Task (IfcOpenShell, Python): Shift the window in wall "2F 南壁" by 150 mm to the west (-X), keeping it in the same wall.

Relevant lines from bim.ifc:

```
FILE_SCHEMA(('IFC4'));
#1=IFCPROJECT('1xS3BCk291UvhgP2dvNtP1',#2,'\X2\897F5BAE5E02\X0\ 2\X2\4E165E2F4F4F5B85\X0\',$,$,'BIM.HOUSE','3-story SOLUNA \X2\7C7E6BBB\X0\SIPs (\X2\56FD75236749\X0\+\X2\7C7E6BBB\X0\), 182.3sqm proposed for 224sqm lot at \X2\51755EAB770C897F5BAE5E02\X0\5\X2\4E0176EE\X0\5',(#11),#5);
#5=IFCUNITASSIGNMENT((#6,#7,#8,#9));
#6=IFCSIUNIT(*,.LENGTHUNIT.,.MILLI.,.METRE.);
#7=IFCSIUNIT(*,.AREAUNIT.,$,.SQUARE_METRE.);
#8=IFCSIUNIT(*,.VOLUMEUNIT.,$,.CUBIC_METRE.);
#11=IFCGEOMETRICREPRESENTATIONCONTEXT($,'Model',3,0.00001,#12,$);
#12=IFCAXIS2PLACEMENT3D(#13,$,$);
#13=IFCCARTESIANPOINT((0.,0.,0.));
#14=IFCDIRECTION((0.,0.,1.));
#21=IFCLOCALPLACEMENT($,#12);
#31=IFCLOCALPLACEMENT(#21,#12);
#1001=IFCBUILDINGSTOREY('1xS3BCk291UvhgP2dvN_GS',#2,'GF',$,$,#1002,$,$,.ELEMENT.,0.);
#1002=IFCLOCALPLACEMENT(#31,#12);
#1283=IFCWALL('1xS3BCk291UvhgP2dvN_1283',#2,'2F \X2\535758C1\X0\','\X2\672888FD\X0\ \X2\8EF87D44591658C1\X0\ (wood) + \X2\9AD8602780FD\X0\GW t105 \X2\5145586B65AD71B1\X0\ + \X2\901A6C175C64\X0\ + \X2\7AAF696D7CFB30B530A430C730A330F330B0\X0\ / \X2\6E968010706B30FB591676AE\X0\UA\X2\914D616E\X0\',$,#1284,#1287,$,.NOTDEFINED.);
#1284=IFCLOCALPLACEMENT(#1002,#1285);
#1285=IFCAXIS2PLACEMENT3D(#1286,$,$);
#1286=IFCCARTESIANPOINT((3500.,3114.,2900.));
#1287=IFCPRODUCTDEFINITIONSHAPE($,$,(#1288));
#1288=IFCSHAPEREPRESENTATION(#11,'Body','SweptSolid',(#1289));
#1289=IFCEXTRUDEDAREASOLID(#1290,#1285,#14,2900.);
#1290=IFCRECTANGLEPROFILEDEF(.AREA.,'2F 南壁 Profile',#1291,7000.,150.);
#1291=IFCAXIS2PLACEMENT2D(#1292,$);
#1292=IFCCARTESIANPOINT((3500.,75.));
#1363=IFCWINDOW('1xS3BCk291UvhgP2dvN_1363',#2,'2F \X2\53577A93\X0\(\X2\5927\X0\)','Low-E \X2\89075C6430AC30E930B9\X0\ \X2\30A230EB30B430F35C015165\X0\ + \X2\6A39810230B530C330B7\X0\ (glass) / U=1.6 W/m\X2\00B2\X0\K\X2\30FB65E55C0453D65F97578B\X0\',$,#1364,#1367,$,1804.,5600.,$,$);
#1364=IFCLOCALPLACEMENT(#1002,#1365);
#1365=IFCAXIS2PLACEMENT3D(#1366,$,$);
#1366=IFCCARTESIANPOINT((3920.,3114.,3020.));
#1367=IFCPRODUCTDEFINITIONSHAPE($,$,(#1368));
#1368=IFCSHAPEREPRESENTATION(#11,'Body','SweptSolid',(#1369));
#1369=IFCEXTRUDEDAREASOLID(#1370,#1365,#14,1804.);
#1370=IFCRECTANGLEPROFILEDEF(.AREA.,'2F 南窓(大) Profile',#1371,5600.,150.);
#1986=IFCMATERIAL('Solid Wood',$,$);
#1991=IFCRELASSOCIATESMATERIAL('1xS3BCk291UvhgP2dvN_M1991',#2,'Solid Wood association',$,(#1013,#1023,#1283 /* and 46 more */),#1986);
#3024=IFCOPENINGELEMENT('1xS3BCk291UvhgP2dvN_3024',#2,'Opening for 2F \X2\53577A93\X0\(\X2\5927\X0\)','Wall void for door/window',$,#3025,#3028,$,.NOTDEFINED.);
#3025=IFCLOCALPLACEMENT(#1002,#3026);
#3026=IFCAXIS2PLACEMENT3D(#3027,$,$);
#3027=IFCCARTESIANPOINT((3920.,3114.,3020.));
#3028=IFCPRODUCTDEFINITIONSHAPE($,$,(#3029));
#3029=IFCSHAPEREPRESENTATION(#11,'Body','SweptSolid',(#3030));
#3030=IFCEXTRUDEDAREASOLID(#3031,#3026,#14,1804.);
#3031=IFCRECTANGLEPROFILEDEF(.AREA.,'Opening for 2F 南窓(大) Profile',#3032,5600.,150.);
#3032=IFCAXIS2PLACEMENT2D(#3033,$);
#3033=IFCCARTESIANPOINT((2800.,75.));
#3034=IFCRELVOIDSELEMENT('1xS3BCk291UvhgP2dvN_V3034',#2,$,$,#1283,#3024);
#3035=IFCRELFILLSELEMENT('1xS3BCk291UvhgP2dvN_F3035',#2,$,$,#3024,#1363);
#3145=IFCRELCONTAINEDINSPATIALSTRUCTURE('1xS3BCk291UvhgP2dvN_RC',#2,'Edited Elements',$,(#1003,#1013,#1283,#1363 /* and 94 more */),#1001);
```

```python
import ifcopenshell
import ifcopenshell.api.geometry
import ifcopenshell.util.placement
import ifcopenshell.util.unit

model = ifcopenshell.open("bim.ifc")
unit_scale = ifcopenshell.util.unit.calculate_unit_scale(model)

window = model.by_id(1363)
opening = window.FillsVoids[0].RelatingOpeningElement
wall = opening.VoidsElements[0].RelatingBuildingElement

wall_matrix = ifcopenshell.util.placement.get_local_placement(wall.ObjectPlacement)
shift = wall_matrix[:3, 0] * -0.15 / unit_scale
before = ifcopenshell.util.placement.get_local_placement(window.ObjectPlacement)[:3, 3].copy()

# The window is not placed relative to its opening, so move both.
for product in (opening, window):
    matrix = ifcopenshell.util.placement.get_local_placement(product.ObjectPlacement)
    matrix[:3, 3] += shift
    ifcopenshell.api.geometry.edit_object_placement(model, product=product, matrix=matrix, is_si=False)

after = ifcopenshell.util.placement.get_local_placement(window.ObjectPlacement)[:3, 3]
print("window moved by", (after - before).round(3) + 0.0)

model.write("bim-out.ifc")
```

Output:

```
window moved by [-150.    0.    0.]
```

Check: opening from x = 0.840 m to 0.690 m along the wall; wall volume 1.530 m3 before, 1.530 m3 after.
